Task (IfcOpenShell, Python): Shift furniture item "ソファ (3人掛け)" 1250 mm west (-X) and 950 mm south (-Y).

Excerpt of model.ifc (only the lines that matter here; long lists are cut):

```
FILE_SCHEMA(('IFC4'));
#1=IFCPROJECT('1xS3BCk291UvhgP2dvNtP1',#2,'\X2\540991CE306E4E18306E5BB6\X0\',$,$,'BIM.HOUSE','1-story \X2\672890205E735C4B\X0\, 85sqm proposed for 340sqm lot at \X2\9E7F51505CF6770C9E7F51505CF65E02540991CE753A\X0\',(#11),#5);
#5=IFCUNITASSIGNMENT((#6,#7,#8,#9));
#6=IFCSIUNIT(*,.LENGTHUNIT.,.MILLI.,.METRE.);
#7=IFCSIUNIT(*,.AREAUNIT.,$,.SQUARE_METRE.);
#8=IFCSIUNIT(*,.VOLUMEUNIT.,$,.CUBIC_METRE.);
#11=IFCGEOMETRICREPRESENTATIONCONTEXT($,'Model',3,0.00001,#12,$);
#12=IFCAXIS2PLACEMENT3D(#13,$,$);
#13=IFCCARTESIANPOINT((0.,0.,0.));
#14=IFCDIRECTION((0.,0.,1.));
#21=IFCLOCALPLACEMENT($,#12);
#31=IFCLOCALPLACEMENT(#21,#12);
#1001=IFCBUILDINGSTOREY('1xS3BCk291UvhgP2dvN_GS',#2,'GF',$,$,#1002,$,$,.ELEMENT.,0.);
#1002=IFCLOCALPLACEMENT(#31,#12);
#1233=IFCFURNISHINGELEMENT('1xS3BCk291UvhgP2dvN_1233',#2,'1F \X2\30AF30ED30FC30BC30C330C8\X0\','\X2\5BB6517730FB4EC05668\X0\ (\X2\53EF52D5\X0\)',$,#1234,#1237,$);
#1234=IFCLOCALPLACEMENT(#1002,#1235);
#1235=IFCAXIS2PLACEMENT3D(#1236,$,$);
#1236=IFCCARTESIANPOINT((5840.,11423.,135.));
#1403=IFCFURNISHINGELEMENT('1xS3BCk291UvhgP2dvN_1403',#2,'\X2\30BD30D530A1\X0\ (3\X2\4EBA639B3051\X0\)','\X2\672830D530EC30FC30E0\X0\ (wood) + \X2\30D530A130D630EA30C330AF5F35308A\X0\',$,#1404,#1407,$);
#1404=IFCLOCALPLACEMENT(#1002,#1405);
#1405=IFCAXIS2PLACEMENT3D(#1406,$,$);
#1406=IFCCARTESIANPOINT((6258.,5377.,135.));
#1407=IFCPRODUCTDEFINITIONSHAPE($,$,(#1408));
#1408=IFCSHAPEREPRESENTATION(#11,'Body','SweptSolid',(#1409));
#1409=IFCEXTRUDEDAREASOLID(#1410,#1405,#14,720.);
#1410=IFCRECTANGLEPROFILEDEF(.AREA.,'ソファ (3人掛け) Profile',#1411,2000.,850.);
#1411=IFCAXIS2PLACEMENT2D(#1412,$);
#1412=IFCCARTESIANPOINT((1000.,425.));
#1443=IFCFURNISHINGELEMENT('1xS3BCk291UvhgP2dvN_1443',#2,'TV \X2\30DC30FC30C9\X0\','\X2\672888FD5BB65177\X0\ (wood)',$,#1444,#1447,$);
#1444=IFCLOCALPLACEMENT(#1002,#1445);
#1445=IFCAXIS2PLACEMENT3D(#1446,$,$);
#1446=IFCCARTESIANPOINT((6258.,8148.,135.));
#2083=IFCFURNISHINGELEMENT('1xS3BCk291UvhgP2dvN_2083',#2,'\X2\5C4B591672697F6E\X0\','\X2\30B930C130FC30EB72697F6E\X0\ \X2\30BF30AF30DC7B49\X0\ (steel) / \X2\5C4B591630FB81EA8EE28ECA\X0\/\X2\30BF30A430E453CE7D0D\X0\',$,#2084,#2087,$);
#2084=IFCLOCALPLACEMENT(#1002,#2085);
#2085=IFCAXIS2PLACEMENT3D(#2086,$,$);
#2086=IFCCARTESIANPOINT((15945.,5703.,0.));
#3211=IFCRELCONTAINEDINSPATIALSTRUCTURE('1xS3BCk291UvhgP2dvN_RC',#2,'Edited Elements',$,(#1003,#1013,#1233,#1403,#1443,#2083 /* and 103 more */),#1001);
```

```python
import ifcopenshell
import ifcopenshell.api.geometry
import ifcopenshell.util.placement

model = ifcopenshell.open("model.ifc")

item = model.by_id(1403)
matrix = ifcopenshell.util.placement.get_local_placement(item.ObjectPlacement)
matrix[0, 3] -= 1250.0
matrix[1, 3] -= 950.0
ifcopenshell.api.geometry.edit_object_placement(model, product=item, matrix=matrix, is_si=False)

print(ifcopenshell.util.placement.get_local_placement(item.ObjectPlacement).round(3) + 0.0)

model.write("model_edited.ifc")
```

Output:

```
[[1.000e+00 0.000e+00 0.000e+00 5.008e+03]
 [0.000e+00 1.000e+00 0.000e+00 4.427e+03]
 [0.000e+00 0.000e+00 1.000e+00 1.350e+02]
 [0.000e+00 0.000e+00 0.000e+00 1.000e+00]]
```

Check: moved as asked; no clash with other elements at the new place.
